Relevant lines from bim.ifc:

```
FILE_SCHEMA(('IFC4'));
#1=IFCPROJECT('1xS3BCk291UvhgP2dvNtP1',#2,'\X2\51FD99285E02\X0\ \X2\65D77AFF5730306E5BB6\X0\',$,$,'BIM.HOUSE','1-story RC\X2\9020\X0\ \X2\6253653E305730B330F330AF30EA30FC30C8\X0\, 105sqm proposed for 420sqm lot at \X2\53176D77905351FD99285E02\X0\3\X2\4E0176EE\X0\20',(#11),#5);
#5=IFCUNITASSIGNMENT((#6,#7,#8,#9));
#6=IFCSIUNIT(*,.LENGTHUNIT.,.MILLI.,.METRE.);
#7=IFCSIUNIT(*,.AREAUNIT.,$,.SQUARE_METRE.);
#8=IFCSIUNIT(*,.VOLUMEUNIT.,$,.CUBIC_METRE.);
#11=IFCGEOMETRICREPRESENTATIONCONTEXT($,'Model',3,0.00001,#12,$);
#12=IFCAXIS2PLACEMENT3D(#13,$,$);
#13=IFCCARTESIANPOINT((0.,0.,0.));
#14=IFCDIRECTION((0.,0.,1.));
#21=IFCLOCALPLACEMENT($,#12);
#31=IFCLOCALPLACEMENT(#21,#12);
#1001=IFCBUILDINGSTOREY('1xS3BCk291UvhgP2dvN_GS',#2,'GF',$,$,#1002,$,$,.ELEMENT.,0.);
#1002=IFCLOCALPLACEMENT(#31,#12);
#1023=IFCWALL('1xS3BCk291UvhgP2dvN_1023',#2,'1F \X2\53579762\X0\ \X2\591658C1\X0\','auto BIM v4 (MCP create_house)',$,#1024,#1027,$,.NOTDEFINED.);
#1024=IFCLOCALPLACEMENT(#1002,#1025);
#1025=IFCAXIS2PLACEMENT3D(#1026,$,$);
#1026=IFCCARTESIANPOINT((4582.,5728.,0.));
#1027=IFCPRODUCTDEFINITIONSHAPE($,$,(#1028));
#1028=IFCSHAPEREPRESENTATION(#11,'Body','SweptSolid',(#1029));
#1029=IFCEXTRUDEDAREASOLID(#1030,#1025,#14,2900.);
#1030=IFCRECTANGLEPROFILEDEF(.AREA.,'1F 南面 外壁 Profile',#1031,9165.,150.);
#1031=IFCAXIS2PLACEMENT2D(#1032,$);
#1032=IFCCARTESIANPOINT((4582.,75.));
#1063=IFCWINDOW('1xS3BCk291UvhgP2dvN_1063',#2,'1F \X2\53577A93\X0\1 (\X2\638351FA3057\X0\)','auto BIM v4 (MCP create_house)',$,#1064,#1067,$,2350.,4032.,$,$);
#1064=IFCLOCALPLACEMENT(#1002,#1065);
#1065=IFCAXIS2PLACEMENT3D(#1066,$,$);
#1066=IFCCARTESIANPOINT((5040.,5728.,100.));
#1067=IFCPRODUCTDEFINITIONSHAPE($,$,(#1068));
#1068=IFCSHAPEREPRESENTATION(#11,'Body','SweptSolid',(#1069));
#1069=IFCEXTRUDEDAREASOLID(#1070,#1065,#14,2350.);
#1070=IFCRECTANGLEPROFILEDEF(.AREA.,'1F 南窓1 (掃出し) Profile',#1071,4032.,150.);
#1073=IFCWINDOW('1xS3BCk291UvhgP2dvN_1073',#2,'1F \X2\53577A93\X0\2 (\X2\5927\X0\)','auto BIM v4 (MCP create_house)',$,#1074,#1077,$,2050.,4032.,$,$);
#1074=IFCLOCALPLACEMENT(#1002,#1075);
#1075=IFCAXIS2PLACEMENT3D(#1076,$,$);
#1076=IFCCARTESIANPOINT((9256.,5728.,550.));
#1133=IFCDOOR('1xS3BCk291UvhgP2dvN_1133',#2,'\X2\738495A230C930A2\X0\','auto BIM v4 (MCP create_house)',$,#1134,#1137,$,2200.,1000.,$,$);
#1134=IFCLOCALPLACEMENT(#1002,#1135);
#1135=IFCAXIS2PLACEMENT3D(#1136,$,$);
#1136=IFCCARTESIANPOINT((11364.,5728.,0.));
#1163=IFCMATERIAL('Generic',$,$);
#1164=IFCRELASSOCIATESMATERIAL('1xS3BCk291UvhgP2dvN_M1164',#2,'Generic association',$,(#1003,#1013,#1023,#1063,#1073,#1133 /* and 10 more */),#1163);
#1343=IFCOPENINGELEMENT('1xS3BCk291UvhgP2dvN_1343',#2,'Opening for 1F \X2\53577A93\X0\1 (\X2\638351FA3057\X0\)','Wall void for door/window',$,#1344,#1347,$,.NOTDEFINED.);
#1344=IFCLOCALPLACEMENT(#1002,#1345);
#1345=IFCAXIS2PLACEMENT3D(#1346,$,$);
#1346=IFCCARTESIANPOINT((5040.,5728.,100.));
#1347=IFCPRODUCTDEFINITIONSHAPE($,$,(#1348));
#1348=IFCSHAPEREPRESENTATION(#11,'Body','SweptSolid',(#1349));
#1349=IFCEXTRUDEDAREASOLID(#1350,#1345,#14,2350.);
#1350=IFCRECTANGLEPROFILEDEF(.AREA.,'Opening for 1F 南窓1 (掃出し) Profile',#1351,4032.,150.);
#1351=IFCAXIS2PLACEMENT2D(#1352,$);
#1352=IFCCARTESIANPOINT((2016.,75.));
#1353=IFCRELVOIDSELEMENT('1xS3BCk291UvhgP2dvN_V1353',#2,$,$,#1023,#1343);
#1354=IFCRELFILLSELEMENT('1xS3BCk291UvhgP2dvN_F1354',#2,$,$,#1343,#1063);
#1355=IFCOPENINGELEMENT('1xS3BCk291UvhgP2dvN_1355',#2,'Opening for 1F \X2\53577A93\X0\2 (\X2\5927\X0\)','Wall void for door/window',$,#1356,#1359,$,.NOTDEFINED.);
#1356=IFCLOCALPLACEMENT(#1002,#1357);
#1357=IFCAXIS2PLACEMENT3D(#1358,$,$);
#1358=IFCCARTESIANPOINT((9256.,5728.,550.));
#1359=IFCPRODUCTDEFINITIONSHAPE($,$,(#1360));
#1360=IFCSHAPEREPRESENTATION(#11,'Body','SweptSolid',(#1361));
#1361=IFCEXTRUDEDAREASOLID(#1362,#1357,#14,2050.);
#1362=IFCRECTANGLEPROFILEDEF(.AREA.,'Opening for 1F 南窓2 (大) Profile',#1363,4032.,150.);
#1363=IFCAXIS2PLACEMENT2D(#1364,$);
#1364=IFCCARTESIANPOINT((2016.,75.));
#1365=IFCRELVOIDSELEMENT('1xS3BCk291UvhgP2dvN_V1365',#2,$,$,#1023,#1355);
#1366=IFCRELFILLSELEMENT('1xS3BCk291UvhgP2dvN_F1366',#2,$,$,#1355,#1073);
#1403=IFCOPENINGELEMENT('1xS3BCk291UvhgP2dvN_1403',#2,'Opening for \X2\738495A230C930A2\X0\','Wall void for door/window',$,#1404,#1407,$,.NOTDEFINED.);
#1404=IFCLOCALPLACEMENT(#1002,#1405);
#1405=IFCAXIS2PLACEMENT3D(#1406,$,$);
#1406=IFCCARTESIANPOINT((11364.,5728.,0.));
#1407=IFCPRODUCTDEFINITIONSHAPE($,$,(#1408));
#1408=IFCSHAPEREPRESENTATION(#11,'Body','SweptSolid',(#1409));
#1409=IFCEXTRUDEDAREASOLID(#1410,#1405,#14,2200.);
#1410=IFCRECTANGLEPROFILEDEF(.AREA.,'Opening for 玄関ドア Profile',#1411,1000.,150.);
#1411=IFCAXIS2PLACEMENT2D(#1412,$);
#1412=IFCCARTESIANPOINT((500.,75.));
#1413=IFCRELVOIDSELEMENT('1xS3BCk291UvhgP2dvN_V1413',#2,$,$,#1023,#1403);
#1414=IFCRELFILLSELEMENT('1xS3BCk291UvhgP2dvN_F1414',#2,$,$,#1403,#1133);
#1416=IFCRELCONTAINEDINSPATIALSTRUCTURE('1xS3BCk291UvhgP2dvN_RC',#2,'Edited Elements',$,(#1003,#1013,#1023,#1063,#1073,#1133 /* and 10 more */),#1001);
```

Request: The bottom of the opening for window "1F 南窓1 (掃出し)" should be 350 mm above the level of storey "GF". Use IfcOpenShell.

```python
import numpy as np
import ifcopenshell
import ifcopenshell.api.geometry
import ifcopenshell.geom
import ifcopenshell.util.element
import ifcopenshell.util.placement
import ifcopenshell.util.shape
import ifcopenshell.util.unit

model = ifcopenshell.open("bim.ifc")
unit_scale = ifcopenshell.util.unit.calculate_unit_scale(model)

window = model.by_guid("1xS3BCk291UvhgP2dvN_1063")
opening = window.FillsVoids[0].RelatingOpeningElement
storey = ifcopenshell.util.element.get_container(window, ifc_class="IfcBuildingStorey")
level = ifcopenshell.util.placement.get_local_placement(storey.ObjectPlacement)[2, 3]

# The opening's origin need not be at the sill, so measure its lowest point.
shape = ifcopenshell.geom.create_shape(ifcopenshell.geom.settings(), opening)
bottom = ifcopenshell.util.shape.get_shape_bottom_elevation(shape, shape.geometry) / unit_scale
dz = level + 350.0 - bottom

shift = np.array([0.0, 0.0, dz])
# The window is not placed relative to its opening, so move both.
for product in (opening, window):
    matrix = ifcopenshell.util.placement.get_local_placement(product.ObjectPlacement)
    matrix[:3, 3] += shift
    ifcopenshell.api.geometry.edit_object_placement(model, product=product, matrix=matrix, is_si=False)

print(f"moved by {dz * unit_scale:+.3f} m")

model.write("bim_v2.ifc")
```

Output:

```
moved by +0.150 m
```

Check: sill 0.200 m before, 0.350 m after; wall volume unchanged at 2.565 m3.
